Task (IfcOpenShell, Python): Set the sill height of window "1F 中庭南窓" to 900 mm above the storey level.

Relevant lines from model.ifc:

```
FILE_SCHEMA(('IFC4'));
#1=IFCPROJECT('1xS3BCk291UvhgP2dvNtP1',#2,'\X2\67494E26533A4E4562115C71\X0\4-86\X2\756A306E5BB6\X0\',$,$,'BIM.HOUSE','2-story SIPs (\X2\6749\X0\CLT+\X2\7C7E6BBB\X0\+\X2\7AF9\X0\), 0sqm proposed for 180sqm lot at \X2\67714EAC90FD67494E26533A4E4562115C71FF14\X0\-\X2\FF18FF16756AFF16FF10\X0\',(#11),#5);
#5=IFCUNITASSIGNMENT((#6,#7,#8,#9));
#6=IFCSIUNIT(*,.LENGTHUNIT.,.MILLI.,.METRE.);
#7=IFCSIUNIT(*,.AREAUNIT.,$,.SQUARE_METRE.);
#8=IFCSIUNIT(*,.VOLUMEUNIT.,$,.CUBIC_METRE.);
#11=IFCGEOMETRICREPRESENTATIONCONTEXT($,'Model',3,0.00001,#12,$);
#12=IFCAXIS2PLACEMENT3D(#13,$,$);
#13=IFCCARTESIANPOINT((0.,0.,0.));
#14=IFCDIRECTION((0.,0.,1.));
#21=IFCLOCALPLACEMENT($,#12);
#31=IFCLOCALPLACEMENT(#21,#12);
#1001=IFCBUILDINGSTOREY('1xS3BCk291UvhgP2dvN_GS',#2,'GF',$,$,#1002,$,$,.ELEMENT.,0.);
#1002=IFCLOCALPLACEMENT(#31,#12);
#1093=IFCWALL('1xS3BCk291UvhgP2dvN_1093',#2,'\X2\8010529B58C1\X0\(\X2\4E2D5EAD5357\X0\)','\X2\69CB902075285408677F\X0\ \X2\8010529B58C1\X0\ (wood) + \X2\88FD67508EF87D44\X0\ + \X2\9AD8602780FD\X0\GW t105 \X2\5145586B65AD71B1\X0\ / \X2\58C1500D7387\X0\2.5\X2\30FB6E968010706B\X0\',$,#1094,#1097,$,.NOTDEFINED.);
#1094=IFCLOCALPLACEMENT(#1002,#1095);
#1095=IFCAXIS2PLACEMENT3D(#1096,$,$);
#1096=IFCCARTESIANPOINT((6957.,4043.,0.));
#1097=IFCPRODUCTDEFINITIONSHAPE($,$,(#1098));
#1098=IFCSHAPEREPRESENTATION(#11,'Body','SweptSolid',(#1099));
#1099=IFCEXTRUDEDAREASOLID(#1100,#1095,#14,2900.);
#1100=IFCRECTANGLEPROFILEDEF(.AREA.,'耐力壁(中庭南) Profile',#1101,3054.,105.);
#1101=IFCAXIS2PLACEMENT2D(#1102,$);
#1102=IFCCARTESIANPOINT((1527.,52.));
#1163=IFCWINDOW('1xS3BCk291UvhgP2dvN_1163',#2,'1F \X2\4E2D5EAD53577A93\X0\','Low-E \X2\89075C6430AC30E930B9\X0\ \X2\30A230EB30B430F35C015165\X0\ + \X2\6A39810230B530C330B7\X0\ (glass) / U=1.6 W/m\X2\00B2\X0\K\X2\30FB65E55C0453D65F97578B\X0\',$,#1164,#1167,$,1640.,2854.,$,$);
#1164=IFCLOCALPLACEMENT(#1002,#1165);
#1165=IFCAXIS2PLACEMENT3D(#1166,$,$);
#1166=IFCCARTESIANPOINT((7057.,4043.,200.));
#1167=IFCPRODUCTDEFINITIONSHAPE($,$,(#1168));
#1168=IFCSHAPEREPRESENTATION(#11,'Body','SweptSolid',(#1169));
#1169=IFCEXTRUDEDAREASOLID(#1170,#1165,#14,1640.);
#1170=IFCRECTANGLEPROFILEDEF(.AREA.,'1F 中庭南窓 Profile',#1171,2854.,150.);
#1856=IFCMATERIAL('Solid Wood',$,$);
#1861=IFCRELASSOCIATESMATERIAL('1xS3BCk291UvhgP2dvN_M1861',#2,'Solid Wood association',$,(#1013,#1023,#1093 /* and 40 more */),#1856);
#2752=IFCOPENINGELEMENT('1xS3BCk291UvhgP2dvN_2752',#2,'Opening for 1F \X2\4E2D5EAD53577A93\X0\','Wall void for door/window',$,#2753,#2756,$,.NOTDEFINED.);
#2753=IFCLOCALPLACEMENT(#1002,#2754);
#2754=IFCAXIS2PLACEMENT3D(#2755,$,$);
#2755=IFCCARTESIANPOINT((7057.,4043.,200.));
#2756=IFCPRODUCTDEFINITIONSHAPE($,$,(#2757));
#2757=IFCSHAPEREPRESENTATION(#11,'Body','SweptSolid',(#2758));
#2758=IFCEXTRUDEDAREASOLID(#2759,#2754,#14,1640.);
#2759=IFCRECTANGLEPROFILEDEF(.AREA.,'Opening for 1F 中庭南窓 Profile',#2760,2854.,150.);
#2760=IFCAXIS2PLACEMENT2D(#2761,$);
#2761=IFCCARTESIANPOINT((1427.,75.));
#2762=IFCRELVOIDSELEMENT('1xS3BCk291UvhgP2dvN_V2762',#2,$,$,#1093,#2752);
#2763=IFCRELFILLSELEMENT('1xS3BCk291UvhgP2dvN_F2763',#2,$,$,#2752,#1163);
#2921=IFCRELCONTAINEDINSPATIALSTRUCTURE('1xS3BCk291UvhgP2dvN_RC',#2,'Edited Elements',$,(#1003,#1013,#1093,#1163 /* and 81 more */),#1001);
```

```python
import numpy as np
import ifcopenshell
import ifcopenshell.api.geometry
import ifcopenshell.geom
import ifcopenshell.util.element
import ifcopenshell.util.placement
import ifcopenshell.util.shape
import ifcopenshell.util.unit

model = ifcopenshell.open("model.ifc")
unit_scale = ifcopenshell.util.unit.calculate_unit_scale(model)

window = model.by_guid("1xS3BCk291UvhgP2dvN_1163")
opening = window.FillsVoids[0].RelatingOpeningElement
storey = ifcopenshell.util.element.get_container(window, ifc_class="IfcBuildingStorey")
level = ifcopenshell.util.placement.get_local_placement(storey.ObjectPlacement)[2, 3]

# The opening's origin need not be at the sill, so measure its lowest point.
shape = ifcopenshell.geom.create_shape(ifcopenshell.geom.settings(), opening)
bottom = ifcopenshell.util.shape.get_shape_bottom_elevation(shape, shape.geometry) / unit_scale
dz = level + 0.9 / unit_scale - bottom

shift = np.array([0.0, 0.0, dz])
# The window is not placed relative to its opening, so move both.
for product in (opening, window):
    matrix = ifcopenshell.util.placement.get_local_placement(product.ObjectPlacement)
    matrix[:3, 3] += shift
    ifcopenshell.api.geometry.edit_object_placement(model, product=product, matrix=matrix, is_si=False)

print(f"moved by {dz * unit_scale:+.3f} m")

model.write("model_edited.ifc")
```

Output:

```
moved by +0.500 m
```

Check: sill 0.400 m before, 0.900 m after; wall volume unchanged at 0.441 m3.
